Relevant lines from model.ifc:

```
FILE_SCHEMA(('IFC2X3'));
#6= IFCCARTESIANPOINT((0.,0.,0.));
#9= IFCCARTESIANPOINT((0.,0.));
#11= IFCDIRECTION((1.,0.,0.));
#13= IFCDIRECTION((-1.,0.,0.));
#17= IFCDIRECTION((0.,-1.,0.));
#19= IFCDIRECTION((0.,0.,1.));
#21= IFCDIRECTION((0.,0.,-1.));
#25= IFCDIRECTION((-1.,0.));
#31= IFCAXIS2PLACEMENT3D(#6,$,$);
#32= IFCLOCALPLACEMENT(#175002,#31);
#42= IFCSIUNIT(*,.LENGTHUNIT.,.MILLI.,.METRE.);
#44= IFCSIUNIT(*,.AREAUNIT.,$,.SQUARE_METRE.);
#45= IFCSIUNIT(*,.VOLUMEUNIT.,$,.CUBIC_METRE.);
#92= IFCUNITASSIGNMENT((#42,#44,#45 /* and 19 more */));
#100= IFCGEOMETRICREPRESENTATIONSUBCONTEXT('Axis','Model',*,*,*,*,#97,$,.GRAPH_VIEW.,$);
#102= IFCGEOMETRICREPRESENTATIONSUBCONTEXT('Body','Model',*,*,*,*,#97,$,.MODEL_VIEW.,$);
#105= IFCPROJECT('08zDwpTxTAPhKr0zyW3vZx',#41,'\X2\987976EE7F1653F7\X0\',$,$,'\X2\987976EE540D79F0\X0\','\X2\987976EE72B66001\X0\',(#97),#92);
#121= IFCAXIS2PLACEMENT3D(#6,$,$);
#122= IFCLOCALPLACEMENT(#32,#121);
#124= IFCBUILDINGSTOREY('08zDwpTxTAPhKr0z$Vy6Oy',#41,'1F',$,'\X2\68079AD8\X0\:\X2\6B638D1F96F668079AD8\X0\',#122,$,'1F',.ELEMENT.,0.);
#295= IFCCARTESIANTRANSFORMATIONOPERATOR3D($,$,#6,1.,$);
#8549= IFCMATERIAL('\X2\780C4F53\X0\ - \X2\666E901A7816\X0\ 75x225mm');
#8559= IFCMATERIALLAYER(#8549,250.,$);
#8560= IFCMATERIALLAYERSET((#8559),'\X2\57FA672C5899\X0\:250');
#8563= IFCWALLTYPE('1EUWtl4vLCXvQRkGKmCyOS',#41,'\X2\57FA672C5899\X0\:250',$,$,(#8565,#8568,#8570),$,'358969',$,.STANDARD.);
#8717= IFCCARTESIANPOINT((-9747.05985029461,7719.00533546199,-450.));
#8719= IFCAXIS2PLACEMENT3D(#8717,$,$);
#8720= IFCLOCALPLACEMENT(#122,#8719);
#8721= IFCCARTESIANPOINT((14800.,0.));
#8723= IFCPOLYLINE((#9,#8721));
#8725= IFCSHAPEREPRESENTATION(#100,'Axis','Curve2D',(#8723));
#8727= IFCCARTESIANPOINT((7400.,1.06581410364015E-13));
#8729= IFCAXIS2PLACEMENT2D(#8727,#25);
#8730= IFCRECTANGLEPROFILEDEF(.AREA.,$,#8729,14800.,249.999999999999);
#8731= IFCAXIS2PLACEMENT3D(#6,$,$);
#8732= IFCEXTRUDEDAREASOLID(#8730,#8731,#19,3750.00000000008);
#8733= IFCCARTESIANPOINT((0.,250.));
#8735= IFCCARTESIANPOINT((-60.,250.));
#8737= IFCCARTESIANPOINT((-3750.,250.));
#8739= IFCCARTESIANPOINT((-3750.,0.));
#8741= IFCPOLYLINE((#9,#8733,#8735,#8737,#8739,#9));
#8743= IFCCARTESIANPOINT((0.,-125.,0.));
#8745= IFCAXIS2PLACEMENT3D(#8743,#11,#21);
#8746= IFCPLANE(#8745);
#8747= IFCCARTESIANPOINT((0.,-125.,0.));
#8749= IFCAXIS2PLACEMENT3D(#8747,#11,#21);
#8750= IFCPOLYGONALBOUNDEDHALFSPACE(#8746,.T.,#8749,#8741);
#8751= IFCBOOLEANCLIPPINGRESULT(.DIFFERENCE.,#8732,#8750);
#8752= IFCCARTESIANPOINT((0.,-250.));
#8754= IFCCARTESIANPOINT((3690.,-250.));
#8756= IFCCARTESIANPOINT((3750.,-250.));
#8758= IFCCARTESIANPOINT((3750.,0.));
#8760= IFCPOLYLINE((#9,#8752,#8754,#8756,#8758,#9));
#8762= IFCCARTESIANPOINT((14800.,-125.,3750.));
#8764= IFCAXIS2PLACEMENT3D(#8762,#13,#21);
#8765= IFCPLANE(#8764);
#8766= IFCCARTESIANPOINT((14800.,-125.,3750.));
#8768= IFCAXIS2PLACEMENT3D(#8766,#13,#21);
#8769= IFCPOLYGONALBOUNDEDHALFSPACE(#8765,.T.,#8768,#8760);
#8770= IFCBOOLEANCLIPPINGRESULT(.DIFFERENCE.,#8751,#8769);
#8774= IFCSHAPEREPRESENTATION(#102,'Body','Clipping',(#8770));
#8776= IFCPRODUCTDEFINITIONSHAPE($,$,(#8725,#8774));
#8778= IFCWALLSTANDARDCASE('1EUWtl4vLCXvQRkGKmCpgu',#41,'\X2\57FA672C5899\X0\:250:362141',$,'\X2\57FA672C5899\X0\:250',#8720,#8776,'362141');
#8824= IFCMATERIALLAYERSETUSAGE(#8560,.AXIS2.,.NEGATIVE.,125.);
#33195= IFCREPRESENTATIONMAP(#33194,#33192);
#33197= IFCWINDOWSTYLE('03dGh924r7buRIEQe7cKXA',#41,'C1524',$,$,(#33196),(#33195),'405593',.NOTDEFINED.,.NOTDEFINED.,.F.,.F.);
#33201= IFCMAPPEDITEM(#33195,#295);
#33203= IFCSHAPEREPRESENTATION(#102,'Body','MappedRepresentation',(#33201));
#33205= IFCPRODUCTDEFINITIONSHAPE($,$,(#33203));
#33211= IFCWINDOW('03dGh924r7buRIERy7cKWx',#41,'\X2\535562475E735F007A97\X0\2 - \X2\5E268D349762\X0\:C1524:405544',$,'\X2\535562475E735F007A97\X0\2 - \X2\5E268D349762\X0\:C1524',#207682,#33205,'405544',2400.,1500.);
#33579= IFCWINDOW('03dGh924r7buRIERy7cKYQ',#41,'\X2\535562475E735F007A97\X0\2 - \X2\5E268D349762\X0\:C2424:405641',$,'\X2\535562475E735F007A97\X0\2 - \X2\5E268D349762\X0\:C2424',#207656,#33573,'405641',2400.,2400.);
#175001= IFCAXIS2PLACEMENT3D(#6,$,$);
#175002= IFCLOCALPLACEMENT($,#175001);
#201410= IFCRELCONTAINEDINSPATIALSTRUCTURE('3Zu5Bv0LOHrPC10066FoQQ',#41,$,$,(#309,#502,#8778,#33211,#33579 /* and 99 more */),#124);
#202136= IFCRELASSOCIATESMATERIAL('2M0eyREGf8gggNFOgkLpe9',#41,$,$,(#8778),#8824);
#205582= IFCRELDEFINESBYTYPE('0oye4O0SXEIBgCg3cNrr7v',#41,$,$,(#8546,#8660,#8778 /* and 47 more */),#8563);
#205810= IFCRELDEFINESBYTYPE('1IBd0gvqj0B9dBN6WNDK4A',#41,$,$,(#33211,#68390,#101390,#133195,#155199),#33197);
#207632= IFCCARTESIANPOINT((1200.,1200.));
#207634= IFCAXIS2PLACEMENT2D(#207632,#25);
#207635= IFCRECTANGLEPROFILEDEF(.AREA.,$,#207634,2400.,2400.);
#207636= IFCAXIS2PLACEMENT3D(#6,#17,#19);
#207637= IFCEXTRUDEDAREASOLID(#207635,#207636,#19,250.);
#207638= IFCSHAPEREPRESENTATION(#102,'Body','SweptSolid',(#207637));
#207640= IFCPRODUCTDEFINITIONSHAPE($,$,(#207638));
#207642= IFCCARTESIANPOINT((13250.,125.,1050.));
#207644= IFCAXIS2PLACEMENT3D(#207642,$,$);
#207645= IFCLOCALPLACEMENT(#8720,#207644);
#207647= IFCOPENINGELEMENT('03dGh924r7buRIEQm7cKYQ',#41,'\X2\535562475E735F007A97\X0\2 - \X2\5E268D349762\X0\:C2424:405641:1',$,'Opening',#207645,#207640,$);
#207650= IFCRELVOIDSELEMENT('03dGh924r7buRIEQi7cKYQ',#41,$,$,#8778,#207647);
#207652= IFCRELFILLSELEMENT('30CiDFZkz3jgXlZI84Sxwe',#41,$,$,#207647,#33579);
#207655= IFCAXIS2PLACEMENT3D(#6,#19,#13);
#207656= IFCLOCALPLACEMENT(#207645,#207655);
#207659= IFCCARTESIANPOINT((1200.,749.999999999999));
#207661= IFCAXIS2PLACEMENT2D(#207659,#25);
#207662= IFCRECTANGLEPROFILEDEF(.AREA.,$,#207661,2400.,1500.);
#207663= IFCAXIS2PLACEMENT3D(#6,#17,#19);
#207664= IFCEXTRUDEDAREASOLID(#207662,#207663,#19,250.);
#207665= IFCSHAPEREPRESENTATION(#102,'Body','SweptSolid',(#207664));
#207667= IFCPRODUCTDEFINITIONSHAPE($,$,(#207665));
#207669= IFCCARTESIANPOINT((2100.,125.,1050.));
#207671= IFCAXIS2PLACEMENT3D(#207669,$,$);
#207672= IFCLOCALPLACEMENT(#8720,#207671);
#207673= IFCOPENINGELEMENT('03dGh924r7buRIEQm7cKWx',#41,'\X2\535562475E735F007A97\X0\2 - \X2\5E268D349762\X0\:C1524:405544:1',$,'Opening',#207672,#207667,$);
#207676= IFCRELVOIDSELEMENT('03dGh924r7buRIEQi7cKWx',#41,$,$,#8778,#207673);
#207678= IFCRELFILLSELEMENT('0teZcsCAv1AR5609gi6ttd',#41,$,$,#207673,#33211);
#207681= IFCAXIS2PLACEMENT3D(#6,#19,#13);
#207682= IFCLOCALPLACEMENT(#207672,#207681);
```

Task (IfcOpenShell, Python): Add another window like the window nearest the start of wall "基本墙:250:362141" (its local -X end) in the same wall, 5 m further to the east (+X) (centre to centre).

```python
import ifcopenshell
import ifcopenshell.api.feature
import ifcopenshell.api.geometry
import ifcopenshell.api.root
import ifcopenshell.geom
import ifcopenshell.util.element
import ifcopenshell.util.placement
import ifcopenshell.util.shape
import ifcopenshell.util.unit

model = ifcopenshell.open("model.ifc")
unit_scale = ifcopenshell.util.unit.calculate_unit_scale(model)
settings = ifcopenshell.geom.settings()


def volume(element):
    """Net volume in cubic metres, openings subtracted."""
    shape = ifcopenshell.geom.create_shape(settings, element)
    return ifcopenshell.util.shape.get_volume(shape.geometry)


def reuse_history(source, copy):
    """copy_class also copies each property set's owner history, people and application; keep the originals."""
    for rel in copy.IsDefinedBy:
        if rel.is_a("IfcRelDefinesByProperties") and (history := rel.RelatingPropertyDefinition.OwnerHistory):
            rel.RelatingPropertyDefinition.OwnerHistory = source.OwnerHistory
            ifcopenshell.util.element.remove_deep2(model, history)


window = model.by_guid("03dGh924r7buRIERy7cKWx")
opening = window.FillsVoids[0].RelatingOpeningElement
wall = opening.VoidsElements[0].RelatingBuildingElement
before = volume(wall)
shift = ifcopenshell.util.placement.get_local_placement(wall.ObjectPlacement)[:3, 0] * 5 / unit_scale

# copy_class copies the void relationship, type, container and properties, but no geometry.
new_opening = ifcopenshell.api.root.copy_class(model, product=opening)
new_opening.Representation = ifcopenshell.util.element.copy_deep(
    model, opening.Representation, exclude=["IfcGeometricRepresentationContext", "IfcRepresentationMap"]
)
new_opening.Name = "单扇平开窗2 - 带贴面:C1524"
new_window = ifcopenshell.api.root.copy_class(model, product=window)
new_window.Representation = ifcopenshell.util.element.copy_deep(
    model, window.Representation, exclude=["IfcGeometricRepresentationContext", "IfcRepresentationMap"]
)
new_window.Name = "单扇平开窗2 - 带贴面:C1524"
new_window.Tag = None
reuse_history(window, new_window)
fills = ifcopenshell.api.feature.add_filling(model, opening=new_opening, element=new_window)
fills.OwnerHistory = new_window.OwnerHistory  # required in IFC2X3

for old, new in ((opening, new_opening), (window, new_window)):
    matrix = ifcopenshell.util.placement.get_local_placement(old.ObjectPlacement)
    matrix[:3, 3] += shift
    ifcopenshell.api.geometry.edit_object_placement(model, product=new, matrix=matrix, is_si=False)

after = volume(wall)

print(f"wall volume {before:.3f} -> {after:.3f} m3")

model.write("model-out.ifc")
```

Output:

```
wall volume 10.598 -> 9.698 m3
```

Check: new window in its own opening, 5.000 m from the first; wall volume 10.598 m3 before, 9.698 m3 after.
